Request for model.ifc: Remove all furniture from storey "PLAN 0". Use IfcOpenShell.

First a look at what the model holds.

```python
import ifcopenshell
import ifcopenshell.util.element

model = ifcopenshell.open("model.ifc")
print(model.schema)
storey = next(s for s in model.by_type("IfcBuildingStorey") if s.Name == "PLAN 0")
furniture = [e for e in ifcopenshell.util.element.get_decomposition(storey) if e.is_a("IfcFurnishingElement")]
seen = {}
for e in furniture:
    element_type = ifcopenshell.util.element.get_type(e)
    name = element_type.Name if element_type not in (None, e) else None
    seen[name] = seen.get(name, 0) + 1
for name, count in sorted(seen.items(), key=str):
    print(count, "x", name)
```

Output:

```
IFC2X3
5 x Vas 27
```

```python
import ifcopenshell
import ifcopenshell.api.root
import ifcopenshell.util.element

model = ifcopenshell.open("model.ifc")

storey = next(s for s in model.by_type("IfcBuildingStorey") if s.Name == "PLAN 0")
furniture = [e for e in ifcopenshell.util.element.get_decomposition(storey) if e.is_a("IfcFurnishingElement")]

for e in furniture:
    ifcopenshell.api.root.remove_product(model, product=e)
print(len(furniture), "removed")

model.write("model-out.ifc")
```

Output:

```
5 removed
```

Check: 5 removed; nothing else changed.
